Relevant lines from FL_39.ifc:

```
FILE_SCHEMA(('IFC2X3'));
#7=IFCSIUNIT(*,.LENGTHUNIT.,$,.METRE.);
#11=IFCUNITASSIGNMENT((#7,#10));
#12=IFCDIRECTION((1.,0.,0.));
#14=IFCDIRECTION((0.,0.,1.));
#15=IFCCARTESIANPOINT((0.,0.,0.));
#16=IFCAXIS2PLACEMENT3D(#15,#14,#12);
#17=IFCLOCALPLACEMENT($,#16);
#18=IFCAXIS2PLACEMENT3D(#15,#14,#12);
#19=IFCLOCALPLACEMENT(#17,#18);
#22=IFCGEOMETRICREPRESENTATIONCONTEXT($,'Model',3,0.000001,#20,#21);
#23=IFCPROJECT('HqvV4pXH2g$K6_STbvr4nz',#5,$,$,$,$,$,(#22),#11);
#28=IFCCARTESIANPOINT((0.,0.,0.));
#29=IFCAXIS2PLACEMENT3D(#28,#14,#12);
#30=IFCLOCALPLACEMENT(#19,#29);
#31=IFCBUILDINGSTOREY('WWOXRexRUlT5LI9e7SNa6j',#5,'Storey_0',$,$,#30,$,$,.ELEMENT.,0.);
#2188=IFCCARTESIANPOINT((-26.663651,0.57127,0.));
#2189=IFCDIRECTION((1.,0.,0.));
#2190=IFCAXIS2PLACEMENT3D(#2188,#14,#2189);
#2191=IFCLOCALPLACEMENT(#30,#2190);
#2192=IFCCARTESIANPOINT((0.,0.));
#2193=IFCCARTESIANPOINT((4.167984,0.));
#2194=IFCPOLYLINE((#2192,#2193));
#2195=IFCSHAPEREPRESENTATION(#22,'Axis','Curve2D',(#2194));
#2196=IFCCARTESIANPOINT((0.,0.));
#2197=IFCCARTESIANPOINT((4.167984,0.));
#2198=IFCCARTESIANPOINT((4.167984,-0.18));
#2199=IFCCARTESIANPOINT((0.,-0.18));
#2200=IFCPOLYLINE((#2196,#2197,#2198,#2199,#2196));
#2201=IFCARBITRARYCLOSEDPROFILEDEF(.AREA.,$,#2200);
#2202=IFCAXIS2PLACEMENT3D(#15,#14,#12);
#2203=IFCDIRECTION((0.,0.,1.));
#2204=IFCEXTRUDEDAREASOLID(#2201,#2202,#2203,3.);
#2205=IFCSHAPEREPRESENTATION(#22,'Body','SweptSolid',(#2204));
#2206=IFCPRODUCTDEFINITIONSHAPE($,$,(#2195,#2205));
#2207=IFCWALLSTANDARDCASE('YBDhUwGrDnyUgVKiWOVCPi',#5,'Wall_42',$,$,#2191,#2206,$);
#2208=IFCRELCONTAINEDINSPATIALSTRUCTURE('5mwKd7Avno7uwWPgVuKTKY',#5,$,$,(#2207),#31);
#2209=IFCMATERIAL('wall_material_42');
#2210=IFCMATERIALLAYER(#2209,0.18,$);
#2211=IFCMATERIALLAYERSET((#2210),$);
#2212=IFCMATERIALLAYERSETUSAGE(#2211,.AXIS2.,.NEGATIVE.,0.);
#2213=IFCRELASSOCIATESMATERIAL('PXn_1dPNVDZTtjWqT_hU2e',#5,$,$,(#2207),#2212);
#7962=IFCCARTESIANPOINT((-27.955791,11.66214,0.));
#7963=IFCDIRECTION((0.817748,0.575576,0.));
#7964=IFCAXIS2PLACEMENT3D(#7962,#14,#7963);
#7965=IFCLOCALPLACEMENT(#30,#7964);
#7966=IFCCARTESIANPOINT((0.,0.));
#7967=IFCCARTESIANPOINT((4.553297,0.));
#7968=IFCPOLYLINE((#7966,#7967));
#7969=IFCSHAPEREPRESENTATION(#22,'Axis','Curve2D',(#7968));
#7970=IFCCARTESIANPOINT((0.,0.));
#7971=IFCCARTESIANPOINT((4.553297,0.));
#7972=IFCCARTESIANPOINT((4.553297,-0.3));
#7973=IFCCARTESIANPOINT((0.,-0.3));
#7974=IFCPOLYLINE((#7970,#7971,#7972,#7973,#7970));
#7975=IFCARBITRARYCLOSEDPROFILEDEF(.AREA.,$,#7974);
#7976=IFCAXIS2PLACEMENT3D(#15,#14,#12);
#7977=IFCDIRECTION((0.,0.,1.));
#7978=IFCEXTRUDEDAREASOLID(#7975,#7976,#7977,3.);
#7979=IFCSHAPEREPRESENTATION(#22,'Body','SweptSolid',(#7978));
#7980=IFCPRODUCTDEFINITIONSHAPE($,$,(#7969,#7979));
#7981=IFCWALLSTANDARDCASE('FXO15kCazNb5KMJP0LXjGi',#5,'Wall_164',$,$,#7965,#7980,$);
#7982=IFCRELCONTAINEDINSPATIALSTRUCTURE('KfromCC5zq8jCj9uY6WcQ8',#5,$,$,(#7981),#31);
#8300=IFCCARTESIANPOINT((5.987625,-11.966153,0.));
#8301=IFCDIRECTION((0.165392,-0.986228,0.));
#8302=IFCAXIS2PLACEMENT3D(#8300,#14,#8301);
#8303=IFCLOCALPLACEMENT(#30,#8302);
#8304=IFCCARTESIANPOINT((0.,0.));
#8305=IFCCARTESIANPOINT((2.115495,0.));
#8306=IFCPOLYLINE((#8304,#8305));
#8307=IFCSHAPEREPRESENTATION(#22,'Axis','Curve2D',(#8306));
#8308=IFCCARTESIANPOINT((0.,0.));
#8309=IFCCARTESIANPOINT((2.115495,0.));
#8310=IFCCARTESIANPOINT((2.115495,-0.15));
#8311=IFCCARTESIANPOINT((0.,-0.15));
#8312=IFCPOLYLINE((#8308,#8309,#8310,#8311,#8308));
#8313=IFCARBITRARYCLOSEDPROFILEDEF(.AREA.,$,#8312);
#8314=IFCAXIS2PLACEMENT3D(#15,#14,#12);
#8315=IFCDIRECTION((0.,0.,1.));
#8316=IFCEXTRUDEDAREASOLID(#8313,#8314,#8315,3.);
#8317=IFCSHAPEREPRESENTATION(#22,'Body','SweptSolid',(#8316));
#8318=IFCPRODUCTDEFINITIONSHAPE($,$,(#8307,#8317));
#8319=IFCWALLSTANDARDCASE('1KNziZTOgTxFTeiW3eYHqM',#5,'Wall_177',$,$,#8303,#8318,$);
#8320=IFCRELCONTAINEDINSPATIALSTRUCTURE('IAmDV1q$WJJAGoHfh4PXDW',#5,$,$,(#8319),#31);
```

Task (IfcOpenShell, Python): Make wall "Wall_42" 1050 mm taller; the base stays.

```python
import ifcopenshell
import ifcopenshell.geom
import ifcopenshell.util.shape

model = ifcopenshell.open("FL_39.ifc")
settings = ifcopenshell.geom.settings()


def volume(element):
    """Net volume in cubic metres, openings subtracted."""
    shape = ifcopenshell.geom.create_shape(settings, element)
    return ifcopenshell.util.shape.get_volume(shape.geometry)


wall = model.by_guid("YBDhUwGrDnyUgVKiWOVCPi")
before = volume(wall)

body = next(r for r in wall.Representation.Representations if r.RepresentationIdentifier == "Body")
solid = body.Items[0]
old_height = solid.Depth
solid.Depth += 1.05
after = volume(wall)

print(f"height {old_height:g} -> {solid.Depth:g}, volume {before:.3f} -> {after:.3f} m3")

model.write("FL_39_edited.ifc")
```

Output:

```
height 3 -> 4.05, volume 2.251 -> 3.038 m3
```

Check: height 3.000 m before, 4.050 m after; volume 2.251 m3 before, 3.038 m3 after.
